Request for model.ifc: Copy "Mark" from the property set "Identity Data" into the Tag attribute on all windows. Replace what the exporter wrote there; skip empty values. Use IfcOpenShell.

First a look at what the model holds.

```python
import ifcopenshell
import ifcopenshell.util.element

model = ifcopenshell.open("model.ifc")
print(model.schema)
windows = model.by_type("IfcWindow")
print(len(windows), "windows")
for e in windows[:8]:
    source = ifcopenshell.util.element.get_pset(e, "Identity Data", "Mark")
    target = e.Tag
    print(e.id(), repr(source), repr(target), sep=" | ")
```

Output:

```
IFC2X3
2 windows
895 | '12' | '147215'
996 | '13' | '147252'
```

```python
import ifcopenshell
import ifcopenshell.util.element

model = ifcopenshell.open("model.ifc")

count = 0
for e in model.by_type("IfcWindow"):
    value = ifcopenshell.util.element.get_pset(e, "Identity Data", "Mark")
    current = e.Tag
    if not value or not value.strip() or current == value:
        continue
    e.Tag = value
    count += 1

print(count, "windows updated")

model.write("model_rev.ifc")
```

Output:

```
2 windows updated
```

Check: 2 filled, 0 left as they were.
